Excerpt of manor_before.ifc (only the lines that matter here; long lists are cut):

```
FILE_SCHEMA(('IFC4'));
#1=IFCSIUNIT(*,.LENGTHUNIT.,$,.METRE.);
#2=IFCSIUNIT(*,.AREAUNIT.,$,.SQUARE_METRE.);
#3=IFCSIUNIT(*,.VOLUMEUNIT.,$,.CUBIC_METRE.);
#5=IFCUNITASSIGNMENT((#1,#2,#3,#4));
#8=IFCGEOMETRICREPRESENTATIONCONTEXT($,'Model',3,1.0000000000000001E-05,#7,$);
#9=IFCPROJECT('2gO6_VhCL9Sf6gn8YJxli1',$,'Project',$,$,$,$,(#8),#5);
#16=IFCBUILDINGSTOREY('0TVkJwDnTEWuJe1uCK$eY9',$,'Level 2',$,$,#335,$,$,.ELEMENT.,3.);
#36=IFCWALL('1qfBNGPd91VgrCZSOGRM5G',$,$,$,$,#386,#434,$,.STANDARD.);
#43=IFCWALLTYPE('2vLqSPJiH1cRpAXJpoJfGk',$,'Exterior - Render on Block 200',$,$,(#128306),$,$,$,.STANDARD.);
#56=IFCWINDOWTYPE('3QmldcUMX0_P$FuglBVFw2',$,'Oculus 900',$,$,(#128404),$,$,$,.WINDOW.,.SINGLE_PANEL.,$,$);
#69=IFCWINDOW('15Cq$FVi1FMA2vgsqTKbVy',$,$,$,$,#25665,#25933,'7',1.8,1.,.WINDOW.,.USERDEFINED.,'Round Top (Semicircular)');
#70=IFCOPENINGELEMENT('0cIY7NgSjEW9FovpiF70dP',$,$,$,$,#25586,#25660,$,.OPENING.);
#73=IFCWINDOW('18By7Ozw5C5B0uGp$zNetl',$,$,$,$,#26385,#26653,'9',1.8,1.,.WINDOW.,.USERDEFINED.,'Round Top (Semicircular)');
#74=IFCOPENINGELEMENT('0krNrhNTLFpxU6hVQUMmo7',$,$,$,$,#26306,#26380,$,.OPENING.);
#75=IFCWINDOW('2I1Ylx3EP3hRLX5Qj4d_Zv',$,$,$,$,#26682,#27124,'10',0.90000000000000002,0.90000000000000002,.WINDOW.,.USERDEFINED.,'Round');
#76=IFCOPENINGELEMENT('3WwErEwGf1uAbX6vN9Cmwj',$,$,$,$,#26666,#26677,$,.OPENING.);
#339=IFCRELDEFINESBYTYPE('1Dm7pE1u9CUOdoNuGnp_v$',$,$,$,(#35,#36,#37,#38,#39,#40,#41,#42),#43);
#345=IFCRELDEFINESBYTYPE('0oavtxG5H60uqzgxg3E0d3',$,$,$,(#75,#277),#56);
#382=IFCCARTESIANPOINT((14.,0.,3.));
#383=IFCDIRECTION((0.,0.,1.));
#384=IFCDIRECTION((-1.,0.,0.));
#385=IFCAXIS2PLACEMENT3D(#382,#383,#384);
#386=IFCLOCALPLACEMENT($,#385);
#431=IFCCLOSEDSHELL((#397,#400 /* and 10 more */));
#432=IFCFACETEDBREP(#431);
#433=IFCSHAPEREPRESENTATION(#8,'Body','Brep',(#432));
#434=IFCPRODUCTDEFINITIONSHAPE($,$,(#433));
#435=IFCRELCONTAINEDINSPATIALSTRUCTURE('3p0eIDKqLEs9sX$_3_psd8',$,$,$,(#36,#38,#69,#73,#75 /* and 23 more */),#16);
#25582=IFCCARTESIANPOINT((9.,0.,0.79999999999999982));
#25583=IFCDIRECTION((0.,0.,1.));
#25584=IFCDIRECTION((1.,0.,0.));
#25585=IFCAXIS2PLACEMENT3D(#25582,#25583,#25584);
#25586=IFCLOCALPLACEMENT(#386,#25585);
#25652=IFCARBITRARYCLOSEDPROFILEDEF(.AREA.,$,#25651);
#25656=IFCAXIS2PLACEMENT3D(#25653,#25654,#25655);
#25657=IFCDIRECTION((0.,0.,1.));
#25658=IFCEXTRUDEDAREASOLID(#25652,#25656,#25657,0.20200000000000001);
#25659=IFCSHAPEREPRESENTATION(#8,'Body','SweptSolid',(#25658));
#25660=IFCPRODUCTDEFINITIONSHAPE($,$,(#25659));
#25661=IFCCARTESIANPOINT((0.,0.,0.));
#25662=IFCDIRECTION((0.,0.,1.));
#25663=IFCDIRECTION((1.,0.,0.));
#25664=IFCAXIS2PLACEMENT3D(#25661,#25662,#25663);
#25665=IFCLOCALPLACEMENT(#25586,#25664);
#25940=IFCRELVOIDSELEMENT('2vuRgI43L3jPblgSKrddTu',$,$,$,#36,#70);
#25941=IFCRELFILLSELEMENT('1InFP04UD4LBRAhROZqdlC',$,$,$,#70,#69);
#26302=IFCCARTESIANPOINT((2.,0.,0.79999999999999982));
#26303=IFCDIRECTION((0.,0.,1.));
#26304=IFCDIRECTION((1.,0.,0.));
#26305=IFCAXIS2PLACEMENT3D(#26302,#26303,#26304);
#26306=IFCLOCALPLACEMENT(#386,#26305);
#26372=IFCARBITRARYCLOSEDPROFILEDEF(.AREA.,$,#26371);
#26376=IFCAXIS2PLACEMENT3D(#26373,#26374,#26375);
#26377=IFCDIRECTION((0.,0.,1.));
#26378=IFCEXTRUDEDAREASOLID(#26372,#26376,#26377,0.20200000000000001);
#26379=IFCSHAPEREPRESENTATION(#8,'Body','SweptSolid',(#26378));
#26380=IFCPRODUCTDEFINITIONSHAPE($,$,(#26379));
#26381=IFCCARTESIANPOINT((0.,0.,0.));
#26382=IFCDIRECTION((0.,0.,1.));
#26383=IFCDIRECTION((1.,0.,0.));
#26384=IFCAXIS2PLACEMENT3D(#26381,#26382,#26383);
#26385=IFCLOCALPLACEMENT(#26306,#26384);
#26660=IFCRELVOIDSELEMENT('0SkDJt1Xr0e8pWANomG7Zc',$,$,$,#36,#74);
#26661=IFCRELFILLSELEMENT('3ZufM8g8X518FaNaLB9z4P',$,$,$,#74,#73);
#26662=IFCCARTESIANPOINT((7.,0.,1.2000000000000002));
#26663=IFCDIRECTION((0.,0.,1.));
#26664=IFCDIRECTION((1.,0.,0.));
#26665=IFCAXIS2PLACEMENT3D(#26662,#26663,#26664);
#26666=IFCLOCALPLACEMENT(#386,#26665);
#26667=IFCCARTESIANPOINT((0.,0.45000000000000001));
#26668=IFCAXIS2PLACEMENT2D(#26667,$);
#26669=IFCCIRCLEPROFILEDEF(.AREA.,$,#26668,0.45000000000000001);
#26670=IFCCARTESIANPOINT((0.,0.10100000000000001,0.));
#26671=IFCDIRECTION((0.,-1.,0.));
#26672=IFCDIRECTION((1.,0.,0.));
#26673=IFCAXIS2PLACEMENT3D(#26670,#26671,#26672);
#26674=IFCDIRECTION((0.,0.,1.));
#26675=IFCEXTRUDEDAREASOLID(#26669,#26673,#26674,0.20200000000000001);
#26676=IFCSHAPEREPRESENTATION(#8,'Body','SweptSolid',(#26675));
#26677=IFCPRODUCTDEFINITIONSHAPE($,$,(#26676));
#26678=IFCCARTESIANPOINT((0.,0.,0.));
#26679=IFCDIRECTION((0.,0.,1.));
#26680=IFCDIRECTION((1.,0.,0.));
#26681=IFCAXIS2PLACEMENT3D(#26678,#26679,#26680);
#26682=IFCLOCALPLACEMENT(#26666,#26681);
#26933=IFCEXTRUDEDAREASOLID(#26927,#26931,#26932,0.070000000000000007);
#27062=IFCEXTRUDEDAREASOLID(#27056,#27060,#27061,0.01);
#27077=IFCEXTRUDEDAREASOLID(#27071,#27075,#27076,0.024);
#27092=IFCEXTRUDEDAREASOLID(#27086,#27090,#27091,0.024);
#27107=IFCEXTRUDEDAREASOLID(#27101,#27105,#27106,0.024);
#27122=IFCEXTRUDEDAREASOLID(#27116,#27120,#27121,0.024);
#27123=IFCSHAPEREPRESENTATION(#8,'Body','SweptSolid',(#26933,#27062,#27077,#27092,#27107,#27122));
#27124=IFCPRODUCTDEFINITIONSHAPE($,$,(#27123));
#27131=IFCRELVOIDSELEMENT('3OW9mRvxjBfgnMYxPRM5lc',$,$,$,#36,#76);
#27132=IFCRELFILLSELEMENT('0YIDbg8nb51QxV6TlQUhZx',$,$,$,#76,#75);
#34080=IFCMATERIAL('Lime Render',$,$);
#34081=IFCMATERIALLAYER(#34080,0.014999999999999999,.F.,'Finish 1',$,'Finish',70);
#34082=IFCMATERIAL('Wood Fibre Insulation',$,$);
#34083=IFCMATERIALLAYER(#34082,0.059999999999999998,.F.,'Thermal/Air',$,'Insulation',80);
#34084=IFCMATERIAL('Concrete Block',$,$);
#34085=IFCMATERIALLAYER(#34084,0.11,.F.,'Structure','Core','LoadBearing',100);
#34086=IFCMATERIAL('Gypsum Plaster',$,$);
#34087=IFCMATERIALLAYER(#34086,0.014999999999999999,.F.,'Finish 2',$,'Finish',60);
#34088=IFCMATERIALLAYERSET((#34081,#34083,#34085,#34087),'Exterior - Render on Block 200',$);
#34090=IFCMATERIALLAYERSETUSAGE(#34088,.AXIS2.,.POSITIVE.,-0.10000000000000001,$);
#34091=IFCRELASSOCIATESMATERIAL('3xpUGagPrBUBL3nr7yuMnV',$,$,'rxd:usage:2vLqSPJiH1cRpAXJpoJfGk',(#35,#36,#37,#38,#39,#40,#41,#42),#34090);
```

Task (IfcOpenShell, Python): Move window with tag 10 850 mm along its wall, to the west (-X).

```python
import ifcopenshell
import ifcopenshell.api.geometry
import ifcopenshell.util.placement

model = ifcopenshell.open("manor_before.ifc")

window = model.by_guid("2I1Ylx3EP3hRLX5Qj4d_Zv")
opening = window.FillsVoids[0].RelatingOpeningElement
wall = opening.VoidsElements[0].RelatingBuildingElement

wall_matrix = ifcopenshell.util.placement.get_local_placement(wall.ObjectPlacement)
shift = wall_matrix[:3, 0] * 0.85
before = ifcopenshell.util.placement.get_local_placement(window.ObjectPlacement)[:3, 3].copy()

# The window is placed relative to its opening, so it follows when the opening moves.
matrix = ifcopenshell.util.placement.get_local_placement(opening.ObjectPlacement)
matrix[:3, 3] += shift
ifcopenshell.api.geometry.edit_object_placement(
    model, product=opening, matrix=matrix, is_si=False, should_transform_children=True
)

after = ifcopenshell.util.placement.get_local_placement(window.ObjectPlacement)[:3, 3]
print("window moved by", (after - before).round(3) + 0.0)

model.write("manor_before_rev.ifc")
```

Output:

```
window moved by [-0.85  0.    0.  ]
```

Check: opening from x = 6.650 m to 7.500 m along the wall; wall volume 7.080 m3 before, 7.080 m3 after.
